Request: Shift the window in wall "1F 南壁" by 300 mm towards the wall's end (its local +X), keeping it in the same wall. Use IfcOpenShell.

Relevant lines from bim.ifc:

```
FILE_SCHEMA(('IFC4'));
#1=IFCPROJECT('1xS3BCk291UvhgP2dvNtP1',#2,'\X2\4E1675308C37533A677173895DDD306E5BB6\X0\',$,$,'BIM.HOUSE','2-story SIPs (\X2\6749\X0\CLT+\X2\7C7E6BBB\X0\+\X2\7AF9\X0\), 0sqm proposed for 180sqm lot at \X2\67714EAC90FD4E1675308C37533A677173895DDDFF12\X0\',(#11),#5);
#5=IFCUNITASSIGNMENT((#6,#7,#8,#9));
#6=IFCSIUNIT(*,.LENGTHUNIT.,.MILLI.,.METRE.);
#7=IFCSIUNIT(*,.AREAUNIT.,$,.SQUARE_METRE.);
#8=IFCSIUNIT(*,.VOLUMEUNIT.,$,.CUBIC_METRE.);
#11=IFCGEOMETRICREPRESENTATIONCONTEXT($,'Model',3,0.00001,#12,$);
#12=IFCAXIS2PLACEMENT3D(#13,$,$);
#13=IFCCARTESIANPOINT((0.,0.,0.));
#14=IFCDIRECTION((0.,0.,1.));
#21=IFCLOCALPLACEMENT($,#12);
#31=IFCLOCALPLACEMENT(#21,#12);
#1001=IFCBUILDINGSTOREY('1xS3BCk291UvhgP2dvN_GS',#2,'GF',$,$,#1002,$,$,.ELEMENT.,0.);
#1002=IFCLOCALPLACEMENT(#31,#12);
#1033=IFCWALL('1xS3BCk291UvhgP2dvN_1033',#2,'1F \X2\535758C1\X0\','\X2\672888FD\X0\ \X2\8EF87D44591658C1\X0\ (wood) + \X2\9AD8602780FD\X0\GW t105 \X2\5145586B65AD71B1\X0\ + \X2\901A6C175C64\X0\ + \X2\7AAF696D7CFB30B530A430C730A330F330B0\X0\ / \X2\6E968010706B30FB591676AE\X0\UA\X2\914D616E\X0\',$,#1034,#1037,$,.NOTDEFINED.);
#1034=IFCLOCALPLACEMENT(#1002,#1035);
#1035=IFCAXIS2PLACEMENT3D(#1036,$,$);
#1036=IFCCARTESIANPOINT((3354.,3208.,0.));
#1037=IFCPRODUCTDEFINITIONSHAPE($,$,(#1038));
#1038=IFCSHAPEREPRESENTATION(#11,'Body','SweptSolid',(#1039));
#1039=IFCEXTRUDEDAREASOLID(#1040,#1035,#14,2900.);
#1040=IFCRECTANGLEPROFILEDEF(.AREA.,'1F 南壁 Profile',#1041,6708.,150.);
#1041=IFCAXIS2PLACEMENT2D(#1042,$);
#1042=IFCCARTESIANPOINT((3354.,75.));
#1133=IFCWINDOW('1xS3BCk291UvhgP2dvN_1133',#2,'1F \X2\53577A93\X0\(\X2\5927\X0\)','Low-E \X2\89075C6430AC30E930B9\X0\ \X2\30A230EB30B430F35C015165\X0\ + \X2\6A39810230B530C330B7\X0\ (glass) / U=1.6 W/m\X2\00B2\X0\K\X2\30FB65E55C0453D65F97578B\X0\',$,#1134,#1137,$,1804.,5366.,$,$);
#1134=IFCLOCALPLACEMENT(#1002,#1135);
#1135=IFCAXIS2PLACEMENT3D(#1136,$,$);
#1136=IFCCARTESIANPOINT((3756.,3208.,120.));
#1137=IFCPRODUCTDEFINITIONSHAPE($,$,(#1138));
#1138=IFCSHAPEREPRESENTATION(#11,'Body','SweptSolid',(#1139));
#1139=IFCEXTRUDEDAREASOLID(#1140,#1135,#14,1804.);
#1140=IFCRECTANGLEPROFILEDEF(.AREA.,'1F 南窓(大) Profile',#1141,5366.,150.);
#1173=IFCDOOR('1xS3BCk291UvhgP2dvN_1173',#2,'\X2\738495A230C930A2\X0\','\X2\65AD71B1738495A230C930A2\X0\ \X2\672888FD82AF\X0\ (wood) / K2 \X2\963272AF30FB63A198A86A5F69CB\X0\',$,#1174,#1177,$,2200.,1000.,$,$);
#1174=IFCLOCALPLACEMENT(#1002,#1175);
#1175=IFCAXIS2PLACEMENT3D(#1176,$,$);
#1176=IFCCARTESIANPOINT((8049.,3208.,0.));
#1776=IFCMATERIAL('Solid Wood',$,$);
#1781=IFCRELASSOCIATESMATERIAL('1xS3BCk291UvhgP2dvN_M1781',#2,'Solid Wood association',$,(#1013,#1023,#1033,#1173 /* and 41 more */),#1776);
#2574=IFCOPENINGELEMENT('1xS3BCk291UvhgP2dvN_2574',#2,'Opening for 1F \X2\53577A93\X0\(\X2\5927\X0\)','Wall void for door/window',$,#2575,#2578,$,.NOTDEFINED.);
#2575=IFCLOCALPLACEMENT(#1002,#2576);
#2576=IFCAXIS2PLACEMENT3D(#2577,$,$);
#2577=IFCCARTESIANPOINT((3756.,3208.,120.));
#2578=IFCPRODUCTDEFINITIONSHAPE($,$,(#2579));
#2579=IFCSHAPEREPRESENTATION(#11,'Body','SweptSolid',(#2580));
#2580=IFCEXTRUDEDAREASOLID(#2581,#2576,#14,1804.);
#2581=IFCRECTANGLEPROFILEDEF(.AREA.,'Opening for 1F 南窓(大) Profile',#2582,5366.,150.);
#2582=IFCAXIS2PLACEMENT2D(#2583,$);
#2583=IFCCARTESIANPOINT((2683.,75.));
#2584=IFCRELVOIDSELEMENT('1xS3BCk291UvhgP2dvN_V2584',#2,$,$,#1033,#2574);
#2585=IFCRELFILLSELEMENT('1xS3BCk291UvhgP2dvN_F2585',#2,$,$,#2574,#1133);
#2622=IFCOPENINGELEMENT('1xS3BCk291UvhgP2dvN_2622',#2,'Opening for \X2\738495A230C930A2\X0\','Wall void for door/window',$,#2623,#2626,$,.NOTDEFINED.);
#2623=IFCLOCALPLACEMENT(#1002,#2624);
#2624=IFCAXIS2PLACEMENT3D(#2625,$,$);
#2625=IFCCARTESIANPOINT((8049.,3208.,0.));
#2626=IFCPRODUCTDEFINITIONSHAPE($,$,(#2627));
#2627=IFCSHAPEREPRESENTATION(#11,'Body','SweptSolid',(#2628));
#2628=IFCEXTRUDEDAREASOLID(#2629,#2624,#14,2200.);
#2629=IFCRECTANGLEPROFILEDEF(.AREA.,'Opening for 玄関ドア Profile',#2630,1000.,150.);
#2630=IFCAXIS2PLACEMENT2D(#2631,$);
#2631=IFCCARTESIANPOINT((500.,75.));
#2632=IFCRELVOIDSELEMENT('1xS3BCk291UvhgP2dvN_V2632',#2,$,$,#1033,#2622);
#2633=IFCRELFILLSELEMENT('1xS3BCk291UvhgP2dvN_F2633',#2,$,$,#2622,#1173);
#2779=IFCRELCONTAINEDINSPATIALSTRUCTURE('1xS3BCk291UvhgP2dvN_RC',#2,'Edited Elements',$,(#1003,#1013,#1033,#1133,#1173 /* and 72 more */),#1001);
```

```python
import ifcopenshell
import ifcopenshell.api.geometry
import ifcopenshell.util.placement
import ifcopenshell.util.unit

model = ifcopenshell.open("bim.ifc")
unit_scale = ifcopenshell.util.unit.calculate_unit_scale(model)

window = model.by_guid("1xS3BCk291UvhgP2dvN_1133")
opening = window.FillsVoids[0].RelatingOpeningElement
wall = opening.VoidsElements[0].RelatingBuildingElement

wall_matrix = ifcopenshell.util.placement.get_local_placement(wall.ObjectPlacement)
shift = wall_matrix[:3, 0] * 0.3 / unit_scale
before = ifcopenshell.util.placement.get_local_placement(window.ObjectPlacement)[:3, 3].copy()

# The window is not placed relative to its opening, so move both.
for product in (opening, window):
    matrix = ifcopenshell.util.placement.get_local_placement(product.ObjectPlacement)
    matrix[:3, 3] += shift
    ifcopenshell.api.geometry.edit_object_placement(model, product=product, matrix=matrix, is_si=False)

after = ifcopenshell.util.placement.get_local_placement(window.ObjectPlacement)[:3, 3]
print("window moved by", (after - before).round(3) + 0.0)

model.write("bim-out.ifc")
```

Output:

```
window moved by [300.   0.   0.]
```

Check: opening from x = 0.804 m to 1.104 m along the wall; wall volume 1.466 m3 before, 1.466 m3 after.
